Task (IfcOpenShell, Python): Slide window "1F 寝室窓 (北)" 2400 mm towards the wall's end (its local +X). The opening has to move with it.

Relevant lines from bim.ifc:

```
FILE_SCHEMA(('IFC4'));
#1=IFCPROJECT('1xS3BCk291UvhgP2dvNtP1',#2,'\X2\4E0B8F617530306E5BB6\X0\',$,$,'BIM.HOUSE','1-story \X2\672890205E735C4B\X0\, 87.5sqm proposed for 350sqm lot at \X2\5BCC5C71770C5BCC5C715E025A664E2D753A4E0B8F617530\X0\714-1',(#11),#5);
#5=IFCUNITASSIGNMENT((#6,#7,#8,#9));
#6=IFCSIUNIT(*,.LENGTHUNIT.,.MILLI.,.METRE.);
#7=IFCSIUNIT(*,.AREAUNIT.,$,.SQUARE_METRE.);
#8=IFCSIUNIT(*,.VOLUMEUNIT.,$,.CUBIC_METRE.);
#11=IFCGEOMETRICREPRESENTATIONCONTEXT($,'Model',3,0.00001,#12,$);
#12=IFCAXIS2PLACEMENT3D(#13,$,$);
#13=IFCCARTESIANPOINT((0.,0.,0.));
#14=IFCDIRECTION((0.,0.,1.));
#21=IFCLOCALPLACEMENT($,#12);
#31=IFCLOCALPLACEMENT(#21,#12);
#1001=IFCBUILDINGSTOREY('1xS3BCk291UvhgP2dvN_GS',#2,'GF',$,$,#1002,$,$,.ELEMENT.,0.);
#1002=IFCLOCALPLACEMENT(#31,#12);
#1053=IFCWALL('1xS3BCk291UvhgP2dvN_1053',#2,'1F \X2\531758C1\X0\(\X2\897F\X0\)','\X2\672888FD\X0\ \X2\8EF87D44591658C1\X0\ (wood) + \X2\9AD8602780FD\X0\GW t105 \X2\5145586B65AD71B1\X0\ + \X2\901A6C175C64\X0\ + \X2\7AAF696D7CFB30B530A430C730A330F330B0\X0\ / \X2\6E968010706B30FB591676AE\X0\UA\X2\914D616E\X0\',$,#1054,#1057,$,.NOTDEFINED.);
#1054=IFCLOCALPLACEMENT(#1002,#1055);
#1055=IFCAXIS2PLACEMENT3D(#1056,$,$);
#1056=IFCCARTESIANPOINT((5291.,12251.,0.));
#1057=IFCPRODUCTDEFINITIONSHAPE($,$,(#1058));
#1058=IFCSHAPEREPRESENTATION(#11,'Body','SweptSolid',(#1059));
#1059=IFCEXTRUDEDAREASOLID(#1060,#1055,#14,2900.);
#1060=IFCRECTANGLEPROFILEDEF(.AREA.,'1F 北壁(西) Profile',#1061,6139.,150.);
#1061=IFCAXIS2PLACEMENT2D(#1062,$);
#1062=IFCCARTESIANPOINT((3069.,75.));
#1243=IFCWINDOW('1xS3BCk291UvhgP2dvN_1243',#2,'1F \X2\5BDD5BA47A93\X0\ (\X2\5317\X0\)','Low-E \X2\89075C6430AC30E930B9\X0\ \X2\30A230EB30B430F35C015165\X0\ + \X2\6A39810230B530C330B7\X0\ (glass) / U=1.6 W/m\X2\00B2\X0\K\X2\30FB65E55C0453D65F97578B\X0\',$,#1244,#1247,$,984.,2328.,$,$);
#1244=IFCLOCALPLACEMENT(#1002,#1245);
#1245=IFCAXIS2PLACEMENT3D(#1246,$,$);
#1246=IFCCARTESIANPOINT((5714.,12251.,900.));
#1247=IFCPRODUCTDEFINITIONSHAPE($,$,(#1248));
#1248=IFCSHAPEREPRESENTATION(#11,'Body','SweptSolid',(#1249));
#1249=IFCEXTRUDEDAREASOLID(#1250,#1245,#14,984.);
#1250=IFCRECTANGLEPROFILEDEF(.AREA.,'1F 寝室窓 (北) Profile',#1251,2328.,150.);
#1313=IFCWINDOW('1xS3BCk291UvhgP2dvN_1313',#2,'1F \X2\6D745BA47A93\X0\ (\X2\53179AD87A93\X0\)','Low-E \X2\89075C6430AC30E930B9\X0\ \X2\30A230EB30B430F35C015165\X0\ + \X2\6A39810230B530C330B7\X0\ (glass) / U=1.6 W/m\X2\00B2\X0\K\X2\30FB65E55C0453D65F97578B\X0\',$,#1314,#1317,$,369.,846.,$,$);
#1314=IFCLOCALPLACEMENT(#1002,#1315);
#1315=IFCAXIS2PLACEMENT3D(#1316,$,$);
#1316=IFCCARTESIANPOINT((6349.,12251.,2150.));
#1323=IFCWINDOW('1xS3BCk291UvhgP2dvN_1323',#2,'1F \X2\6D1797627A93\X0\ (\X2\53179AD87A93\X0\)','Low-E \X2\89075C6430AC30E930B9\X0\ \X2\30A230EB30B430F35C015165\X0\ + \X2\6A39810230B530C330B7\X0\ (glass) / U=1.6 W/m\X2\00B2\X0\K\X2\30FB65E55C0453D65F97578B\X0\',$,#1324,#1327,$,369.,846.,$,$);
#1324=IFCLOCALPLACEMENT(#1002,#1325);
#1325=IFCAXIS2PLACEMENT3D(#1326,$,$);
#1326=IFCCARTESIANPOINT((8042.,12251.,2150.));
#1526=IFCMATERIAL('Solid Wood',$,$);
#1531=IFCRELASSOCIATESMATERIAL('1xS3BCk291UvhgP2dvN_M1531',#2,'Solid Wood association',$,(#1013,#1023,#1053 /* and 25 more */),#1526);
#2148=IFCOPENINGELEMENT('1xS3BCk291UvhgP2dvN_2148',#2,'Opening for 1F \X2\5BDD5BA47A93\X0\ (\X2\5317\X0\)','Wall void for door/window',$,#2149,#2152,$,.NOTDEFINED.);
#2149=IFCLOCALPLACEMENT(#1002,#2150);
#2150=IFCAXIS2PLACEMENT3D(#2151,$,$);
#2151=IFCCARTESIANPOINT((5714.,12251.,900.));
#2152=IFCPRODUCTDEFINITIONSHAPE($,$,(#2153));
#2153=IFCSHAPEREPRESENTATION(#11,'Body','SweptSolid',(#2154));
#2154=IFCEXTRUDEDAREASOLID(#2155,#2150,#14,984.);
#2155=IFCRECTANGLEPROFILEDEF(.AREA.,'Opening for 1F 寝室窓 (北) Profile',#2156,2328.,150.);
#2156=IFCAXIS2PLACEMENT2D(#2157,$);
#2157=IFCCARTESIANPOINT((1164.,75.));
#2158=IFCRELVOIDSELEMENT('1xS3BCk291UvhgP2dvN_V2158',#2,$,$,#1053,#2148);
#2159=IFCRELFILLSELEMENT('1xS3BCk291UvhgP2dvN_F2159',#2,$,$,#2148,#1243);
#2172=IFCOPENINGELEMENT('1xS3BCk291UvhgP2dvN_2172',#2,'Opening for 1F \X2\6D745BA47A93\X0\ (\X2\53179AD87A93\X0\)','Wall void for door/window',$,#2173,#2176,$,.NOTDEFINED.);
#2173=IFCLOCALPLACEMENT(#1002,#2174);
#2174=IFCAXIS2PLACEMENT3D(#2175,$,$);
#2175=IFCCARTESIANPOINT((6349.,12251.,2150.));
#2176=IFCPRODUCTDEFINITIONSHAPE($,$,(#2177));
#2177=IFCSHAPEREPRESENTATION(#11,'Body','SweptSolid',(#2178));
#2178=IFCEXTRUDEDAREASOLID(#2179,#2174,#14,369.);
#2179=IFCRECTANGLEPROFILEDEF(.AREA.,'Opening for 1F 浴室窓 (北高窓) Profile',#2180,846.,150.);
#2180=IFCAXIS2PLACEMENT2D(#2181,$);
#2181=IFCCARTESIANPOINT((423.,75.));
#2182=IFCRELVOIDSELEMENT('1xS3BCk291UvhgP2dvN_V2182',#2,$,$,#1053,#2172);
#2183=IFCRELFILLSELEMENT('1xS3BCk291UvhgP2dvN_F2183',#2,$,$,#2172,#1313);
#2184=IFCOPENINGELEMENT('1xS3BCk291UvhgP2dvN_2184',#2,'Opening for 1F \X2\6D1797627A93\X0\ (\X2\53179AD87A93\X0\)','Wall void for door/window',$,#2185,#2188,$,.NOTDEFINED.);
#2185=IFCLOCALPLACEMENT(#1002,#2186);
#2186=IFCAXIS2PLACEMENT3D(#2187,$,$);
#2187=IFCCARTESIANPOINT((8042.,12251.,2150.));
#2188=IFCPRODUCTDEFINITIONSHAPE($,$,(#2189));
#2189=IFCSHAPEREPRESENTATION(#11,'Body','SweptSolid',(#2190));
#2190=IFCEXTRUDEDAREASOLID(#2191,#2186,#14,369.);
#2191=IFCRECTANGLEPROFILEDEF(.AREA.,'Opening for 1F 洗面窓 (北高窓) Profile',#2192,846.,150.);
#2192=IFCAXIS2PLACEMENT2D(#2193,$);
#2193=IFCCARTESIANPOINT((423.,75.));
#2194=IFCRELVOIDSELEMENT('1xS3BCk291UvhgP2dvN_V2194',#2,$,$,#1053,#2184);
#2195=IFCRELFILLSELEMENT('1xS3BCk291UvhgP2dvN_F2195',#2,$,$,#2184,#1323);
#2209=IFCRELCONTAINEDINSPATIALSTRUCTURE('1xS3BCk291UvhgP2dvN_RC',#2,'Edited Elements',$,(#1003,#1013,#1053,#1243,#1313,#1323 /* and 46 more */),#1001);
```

```python
import ifcopenshell
import ifcopenshell.api.geometry
import ifcopenshell.util.placement

model = ifcopenshell.open("bim.ifc")

window = model.by_guid("1xS3BCk291UvhgP2dvN_1243")
opening = window.FillsVoids[0].RelatingOpeningElement
wall = opening.VoidsElements[0].RelatingBuildingElement

wall_matrix = ifcopenshell.util.placement.get_local_placement(wall.ObjectPlacement)
shift = wall_matrix[:3, 0] * 2400.0
before = ifcopenshell.util.placement.get_local_placement(window.ObjectPlacement)[:3, 3].copy()

# The window is not placed relative to its opening, so move both.
for product in (opening, window):
    matrix = ifcopenshell.util.placement.get_local_placement(product.ObjectPlacement)
    matrix[:3, 3] += shift
    ifcopenshell.api.geometry.edit_object_placement(model, product=product, matrix=matrix, is_si=False)

after = ifcopenshell.util.placement.get_local_placement(window.ObjectPlacement)[:3, 3]
print("window moved by", (after - before).round(3) + 0.0)

model.write("bim_rev.ifc")
```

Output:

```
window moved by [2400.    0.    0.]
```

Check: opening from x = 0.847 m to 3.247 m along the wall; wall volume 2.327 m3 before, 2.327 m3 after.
